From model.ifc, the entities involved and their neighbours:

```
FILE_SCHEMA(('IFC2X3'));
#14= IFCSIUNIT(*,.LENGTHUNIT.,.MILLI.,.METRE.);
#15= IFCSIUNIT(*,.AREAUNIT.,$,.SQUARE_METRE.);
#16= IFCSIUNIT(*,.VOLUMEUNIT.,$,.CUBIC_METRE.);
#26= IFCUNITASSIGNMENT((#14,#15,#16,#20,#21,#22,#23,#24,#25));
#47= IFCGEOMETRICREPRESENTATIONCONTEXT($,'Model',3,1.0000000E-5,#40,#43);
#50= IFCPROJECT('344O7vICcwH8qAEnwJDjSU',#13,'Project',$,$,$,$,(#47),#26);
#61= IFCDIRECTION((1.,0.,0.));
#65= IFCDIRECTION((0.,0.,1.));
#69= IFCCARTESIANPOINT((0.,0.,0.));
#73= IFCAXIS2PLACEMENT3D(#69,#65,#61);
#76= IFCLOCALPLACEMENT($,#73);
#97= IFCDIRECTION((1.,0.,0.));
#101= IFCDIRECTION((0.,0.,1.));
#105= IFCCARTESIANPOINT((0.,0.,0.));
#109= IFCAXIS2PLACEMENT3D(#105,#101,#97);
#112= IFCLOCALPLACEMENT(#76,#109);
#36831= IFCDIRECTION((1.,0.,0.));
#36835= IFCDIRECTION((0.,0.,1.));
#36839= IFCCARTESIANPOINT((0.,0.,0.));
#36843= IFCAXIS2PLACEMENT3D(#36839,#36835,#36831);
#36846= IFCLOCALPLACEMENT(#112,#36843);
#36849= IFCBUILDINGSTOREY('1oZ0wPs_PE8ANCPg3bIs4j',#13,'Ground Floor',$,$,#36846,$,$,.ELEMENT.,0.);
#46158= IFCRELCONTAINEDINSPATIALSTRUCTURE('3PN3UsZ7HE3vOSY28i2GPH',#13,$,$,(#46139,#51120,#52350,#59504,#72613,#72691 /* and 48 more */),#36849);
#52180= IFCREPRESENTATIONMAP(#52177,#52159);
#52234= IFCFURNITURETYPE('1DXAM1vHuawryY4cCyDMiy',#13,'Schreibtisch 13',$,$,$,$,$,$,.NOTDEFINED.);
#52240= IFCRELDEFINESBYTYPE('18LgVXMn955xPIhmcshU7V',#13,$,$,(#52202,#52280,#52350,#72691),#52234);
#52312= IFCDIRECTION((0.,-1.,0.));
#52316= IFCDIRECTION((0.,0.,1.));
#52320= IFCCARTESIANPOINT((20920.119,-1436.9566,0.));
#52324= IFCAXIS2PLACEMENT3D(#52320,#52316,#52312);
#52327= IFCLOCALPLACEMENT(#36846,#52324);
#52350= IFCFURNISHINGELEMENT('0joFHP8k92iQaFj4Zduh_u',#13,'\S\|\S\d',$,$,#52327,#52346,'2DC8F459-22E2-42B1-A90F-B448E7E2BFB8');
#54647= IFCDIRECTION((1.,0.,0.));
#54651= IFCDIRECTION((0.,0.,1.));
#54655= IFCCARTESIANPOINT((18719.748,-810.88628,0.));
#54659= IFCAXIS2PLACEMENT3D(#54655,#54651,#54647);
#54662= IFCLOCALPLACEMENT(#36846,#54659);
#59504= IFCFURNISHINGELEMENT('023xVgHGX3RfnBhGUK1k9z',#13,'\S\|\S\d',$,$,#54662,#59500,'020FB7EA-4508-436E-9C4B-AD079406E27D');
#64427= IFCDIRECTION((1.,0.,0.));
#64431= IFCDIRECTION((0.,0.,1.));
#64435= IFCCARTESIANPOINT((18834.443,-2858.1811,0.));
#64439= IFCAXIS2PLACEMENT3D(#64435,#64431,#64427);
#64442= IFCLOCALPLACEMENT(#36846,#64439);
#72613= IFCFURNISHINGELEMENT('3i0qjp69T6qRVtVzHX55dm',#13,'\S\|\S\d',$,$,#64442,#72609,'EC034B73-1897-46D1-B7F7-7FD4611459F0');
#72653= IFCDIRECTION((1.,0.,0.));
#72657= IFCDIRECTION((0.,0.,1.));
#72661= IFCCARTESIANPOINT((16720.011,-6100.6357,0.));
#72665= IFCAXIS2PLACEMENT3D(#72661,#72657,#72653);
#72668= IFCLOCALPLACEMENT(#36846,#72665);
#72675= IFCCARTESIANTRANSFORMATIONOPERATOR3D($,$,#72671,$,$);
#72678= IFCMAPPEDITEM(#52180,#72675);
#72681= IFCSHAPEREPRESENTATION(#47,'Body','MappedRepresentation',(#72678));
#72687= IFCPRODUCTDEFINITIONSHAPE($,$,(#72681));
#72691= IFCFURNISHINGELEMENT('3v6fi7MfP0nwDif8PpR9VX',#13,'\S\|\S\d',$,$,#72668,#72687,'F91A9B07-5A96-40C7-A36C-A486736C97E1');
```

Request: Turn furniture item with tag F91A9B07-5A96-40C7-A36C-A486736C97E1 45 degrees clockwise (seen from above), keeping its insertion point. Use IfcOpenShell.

```python
import ifcopenshell
import ifcopenshell.api.geometry
import ifcopenshell.util.placement

model = ifcopenshell.open("model.ifc")

item = model.by_guid("3v6fi7MfP0nwDif8PpR9VX")
matrix = ifcopenshell.util.placement.get_local_placement(item.ObjectPlacement)
matrix = matrix @ ifcopenshell.util.placement.rotation(-45, "Z")
ifcopenshell.api.geometry.edit_object_placement(model, product=item, matrix=matrix, is_si=False)

print(ifcopenshell.util.placement.get_local_placement(item.ObjectPlacement).round(3) + 0.0)

model.write("model-out.ifc")
```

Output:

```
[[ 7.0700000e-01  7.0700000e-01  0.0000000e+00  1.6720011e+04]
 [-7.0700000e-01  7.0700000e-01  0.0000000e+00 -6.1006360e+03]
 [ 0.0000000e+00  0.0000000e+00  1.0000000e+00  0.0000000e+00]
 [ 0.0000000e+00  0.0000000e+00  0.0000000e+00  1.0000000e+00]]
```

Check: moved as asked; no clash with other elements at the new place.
